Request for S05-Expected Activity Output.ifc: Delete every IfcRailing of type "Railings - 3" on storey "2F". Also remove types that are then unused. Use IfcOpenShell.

First a look at what the model holds.

```python
import ifcopenshell
import ifcopenshell.util.element

model = ifcopenshell.open("S05-Expected Activity Output.ifc")
print(model.schema)
storey = next(s for s in model.by_type("IfcBuildingStorey") if s.Name == "2F")
railings = [e for e in ifcopenshell.util.element.get_decomposition(storey) if e.is_a("IfcRailing")]
seen = {}
for e in railings:
    element_type = ifcopenshell.util.element.get_type(e)
    name = element_type.Name if element_type not in (None, e) else None
    seen[name] = seen.get(name, 0) + 1
for name, count in sorted(seen.items(), key=str):
    print(count, "x", name)
```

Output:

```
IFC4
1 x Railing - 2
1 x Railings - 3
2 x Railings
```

```python
import ifcopenshell
import ifcopenshell.api.root
import ifcopenshell.util.element

model = ifcopenshell.open("S05-Expected Activity Output.ifc")

storey = next(s for s in model.by_type("IfcBuildingStorey") if s.Name == "2F")
railings = [e for e in ifcopenshell.util.element.get_decomposition(storey) if e.is_a("IfcRailing")]
targets = [e for e in railings if (t := ifcopenshell.util.element.get_type(e)) not in (None, e) and t.Name == "Railings - 3"]
types = {ifcopenshell.util.element.get_type(e) for e in targets} - {None, *targets}

for e in targets:
    ifcopenshell.api.root.remove_product(model, product=e)
print(len(targets), "removed")

unused = [t for t in types if not ifcopenshell.util.element.get_types(t)]
for t in unused:
    ifcopenshell.api.root.remove_product(model, product=t)
print(len(unused), "unused types removed")

model.write("S05-Expected Activity Output-out.ifc")
```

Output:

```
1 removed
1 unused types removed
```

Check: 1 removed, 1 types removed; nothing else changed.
